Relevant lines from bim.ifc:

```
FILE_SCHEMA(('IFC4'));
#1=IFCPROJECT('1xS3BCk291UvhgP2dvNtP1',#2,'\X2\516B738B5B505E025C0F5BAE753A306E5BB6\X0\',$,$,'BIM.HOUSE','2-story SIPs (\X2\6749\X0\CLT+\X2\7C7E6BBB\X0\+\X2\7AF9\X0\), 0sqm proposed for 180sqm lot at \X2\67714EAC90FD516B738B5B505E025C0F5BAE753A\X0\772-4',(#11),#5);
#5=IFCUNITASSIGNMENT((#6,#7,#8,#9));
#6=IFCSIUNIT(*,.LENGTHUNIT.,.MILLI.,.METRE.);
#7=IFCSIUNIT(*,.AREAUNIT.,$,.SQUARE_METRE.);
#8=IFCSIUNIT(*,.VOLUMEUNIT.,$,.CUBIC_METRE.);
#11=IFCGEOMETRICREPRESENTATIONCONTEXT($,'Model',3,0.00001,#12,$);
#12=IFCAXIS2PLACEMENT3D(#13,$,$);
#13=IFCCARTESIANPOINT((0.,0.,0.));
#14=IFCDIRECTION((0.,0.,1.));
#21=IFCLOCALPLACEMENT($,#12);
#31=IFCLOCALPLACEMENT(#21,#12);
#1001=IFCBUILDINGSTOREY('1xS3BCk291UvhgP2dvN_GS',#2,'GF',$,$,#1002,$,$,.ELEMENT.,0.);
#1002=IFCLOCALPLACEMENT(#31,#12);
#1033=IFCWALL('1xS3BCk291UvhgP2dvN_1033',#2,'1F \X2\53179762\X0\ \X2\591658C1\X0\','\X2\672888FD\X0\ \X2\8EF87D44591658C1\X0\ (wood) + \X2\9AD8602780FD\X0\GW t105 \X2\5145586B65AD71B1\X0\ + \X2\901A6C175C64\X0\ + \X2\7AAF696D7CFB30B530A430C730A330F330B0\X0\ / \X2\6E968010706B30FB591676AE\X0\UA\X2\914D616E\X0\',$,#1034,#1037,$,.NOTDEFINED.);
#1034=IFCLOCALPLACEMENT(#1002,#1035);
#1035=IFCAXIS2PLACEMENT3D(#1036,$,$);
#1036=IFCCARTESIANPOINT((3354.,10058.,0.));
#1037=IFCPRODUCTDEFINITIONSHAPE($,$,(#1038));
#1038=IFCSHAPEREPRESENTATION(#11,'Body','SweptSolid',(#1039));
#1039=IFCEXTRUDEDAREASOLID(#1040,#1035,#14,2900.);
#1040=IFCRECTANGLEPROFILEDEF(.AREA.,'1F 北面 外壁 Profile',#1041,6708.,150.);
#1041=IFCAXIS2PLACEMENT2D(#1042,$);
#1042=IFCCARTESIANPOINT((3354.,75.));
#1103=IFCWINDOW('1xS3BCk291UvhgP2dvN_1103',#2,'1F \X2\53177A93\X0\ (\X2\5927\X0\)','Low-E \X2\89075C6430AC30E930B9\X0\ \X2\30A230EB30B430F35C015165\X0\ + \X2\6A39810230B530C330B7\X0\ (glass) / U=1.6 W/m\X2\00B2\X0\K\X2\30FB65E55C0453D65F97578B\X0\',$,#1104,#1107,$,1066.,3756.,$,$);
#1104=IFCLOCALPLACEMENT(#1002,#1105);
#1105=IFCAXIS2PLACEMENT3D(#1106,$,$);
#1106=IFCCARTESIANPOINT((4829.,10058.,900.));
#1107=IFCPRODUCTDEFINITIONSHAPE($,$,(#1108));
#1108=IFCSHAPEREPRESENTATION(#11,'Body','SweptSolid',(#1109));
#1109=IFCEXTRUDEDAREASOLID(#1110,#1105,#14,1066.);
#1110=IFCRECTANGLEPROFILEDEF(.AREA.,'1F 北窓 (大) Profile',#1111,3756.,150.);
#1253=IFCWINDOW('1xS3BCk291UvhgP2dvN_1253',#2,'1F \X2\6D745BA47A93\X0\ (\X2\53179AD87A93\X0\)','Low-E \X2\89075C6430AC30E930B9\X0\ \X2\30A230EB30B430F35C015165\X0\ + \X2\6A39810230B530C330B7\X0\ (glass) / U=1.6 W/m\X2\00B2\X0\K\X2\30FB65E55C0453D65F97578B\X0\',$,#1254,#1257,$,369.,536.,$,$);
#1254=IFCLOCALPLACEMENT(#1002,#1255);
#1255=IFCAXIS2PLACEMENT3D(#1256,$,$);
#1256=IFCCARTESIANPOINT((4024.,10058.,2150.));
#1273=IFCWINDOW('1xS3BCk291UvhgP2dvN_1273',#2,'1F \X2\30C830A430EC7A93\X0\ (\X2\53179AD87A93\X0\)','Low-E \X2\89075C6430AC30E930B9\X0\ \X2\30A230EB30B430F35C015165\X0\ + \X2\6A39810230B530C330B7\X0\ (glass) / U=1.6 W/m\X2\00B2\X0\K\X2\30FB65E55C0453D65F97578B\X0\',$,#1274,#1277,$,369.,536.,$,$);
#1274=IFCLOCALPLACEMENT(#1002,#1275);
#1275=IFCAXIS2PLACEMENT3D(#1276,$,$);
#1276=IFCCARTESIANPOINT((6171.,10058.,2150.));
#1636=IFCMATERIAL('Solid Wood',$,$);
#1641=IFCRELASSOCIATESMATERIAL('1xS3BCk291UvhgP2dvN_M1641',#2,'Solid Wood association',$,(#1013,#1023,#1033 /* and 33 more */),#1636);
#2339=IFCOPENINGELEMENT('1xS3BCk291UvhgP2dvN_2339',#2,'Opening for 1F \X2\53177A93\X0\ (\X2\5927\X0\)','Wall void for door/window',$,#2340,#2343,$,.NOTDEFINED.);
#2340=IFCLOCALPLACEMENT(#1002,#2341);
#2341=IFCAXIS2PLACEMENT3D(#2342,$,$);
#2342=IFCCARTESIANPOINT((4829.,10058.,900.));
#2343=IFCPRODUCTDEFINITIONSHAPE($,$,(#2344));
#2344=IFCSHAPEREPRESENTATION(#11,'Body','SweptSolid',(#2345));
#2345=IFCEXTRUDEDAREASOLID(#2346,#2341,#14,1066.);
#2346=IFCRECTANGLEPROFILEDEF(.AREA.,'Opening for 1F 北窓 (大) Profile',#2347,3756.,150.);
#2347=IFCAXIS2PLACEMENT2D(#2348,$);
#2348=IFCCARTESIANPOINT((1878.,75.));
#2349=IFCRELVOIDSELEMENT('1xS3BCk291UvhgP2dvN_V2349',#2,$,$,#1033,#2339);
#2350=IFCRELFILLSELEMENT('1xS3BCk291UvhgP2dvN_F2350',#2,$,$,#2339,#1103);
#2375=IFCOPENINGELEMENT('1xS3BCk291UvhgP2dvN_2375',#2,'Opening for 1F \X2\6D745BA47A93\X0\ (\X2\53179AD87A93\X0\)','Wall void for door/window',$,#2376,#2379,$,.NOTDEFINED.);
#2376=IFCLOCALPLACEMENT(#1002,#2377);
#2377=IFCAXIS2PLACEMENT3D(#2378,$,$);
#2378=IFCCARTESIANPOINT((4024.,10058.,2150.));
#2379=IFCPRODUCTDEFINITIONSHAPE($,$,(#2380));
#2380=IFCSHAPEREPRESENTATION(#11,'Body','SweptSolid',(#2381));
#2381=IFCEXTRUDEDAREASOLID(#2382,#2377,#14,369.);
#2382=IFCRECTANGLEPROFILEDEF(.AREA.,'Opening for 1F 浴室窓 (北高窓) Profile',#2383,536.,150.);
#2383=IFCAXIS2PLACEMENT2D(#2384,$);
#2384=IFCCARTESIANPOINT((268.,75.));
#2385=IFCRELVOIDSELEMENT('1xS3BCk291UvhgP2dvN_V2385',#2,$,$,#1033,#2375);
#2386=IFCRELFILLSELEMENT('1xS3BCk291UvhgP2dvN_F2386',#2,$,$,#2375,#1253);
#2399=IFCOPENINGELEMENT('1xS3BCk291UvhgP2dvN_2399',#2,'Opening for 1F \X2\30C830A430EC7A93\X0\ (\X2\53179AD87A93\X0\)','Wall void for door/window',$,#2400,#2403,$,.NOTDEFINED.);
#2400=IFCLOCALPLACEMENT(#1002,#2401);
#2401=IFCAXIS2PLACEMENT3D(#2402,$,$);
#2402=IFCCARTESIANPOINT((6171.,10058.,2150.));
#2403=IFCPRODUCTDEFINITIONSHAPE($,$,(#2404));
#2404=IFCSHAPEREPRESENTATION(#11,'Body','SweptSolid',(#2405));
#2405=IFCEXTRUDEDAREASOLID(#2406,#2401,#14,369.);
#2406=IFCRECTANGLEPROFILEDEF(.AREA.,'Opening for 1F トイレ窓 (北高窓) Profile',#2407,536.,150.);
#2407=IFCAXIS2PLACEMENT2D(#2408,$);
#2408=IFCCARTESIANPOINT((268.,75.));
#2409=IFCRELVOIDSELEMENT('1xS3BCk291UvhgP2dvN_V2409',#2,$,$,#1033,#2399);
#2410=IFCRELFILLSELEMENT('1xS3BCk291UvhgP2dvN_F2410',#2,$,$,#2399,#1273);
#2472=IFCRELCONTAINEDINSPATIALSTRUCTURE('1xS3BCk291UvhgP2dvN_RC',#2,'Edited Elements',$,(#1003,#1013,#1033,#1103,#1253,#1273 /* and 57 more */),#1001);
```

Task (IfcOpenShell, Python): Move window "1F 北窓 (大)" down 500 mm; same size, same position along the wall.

```python
import numpy as np
import ifcopenshell
import ifcopenshell.api.geometry
import ifcopenshell.util.placement
import ifcopenshell.util.unit

model = ifcopenshell.open("bim.ifc")
unit_scale = ifcopenshell.util.unit.calculate_unit_scale(model)

window = model.by_guid("1xS3BCk291UvhgP2dvN_1103")
opening = window.FillsVoids[0].RelatingOpeningElement
dz = -0.5 / unit_scale

shift = np.array([0.0, 0.0, dz])
# The window is not placed relative to its opening, so move both.
for product in (opening, window):
    matrix = ifcopenshell.util.placement.get_local_placement(product.ObjectPlacement)
    matrix[:3, 3] += shift
    ifcopenshell.api.geometry.edit_object_placement(model, product=product, matrix=matrix, is_si=False)

print(f"moved by {dz * unit_scale:+.3f} m")

model.write("bim_updated.ifc")
```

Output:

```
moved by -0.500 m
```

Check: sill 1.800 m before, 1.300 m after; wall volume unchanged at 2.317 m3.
